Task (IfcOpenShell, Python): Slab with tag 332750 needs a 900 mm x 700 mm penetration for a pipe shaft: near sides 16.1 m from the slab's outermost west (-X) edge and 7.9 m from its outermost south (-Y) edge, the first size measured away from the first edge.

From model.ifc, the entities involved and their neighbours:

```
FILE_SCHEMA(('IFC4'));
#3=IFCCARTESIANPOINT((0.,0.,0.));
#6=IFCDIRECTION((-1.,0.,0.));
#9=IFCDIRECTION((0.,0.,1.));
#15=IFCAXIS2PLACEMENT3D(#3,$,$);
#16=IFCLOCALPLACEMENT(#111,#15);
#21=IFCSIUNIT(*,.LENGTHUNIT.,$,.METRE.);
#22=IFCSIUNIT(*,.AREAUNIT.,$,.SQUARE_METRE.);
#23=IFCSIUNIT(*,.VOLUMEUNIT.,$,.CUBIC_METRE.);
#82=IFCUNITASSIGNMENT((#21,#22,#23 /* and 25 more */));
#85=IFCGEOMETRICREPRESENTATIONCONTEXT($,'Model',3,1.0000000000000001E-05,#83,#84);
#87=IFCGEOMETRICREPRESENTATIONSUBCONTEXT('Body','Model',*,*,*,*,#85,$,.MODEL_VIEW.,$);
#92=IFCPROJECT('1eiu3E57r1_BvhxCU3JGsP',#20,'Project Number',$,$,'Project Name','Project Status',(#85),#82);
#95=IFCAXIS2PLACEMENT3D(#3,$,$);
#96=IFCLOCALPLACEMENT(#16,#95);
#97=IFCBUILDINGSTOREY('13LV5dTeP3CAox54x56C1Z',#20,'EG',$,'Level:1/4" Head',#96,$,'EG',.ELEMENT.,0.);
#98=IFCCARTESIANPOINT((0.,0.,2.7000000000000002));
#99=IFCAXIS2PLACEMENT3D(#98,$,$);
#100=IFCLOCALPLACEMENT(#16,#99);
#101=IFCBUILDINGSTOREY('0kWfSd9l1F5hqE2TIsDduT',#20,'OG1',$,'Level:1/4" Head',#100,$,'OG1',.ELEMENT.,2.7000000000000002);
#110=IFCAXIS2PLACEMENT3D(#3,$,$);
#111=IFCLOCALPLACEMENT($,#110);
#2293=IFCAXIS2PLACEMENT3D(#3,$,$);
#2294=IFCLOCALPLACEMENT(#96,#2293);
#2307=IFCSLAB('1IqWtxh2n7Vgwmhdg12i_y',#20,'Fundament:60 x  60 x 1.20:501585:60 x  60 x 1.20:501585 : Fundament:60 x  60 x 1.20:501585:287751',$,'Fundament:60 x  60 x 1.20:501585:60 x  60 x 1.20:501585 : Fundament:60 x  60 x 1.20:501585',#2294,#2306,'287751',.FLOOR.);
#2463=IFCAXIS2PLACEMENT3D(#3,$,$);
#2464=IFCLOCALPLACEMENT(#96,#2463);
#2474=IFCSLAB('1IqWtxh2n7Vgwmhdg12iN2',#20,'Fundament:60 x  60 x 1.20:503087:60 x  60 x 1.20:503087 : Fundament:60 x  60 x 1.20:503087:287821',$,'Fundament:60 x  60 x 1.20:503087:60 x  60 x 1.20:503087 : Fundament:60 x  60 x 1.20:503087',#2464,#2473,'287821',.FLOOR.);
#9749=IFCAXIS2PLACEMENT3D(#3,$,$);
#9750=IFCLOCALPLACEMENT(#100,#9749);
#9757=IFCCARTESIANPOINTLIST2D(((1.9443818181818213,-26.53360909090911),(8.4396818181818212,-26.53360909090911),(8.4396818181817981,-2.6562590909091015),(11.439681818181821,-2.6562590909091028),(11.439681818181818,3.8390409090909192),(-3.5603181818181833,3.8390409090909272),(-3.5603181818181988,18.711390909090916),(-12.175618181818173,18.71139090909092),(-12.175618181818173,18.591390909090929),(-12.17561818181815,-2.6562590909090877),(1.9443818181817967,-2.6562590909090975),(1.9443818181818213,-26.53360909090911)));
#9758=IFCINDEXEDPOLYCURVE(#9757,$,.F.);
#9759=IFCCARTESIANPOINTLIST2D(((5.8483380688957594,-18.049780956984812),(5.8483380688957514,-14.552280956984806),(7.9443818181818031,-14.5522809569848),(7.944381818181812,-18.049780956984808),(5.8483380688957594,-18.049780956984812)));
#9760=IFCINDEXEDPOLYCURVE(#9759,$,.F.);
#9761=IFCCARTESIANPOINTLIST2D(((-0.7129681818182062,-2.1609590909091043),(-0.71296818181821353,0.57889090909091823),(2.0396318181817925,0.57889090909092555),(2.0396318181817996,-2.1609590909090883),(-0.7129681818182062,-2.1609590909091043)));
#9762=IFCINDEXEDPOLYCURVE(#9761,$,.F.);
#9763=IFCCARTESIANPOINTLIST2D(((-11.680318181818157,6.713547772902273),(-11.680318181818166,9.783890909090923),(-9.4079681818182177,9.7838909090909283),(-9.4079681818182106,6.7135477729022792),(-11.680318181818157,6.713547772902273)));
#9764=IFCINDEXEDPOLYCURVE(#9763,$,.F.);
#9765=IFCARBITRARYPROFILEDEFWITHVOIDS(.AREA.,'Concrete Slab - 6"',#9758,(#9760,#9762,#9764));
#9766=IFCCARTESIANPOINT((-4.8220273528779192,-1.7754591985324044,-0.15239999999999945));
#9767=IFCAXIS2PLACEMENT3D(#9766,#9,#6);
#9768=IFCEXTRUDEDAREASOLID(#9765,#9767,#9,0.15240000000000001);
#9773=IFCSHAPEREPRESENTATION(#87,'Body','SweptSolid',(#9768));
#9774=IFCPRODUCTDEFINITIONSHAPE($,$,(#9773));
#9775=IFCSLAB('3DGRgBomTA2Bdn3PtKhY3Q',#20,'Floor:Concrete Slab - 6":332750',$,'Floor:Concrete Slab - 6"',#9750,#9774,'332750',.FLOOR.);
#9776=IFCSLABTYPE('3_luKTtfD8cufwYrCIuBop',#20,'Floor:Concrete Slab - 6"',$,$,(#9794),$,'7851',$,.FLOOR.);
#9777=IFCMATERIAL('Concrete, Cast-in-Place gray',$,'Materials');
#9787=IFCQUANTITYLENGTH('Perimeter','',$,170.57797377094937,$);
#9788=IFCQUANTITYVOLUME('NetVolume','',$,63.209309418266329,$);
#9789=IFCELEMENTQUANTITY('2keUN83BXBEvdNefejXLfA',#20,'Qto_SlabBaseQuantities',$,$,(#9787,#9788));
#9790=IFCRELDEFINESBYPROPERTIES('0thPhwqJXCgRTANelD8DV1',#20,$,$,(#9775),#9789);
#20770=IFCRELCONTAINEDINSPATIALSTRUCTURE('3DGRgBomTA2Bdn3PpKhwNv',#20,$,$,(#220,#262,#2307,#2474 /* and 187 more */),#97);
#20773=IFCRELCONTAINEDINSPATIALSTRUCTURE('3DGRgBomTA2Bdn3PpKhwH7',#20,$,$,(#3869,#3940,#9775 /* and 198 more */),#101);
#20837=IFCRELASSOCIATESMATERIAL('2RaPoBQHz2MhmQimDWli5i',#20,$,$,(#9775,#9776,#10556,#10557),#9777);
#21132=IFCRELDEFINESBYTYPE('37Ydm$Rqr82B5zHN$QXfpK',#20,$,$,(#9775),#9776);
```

```python
import numpy as np
import ifcopenshell
import ifcopenshell.api.feature
import ifcopenshell.api.geometry
import ifcopenshell.api.pset
import ifcopenshell.api.root
import ifcopenshell.geom
import ifcopenshell.util.element
import ifcopenshell.util.placement
import ifcopenshell.util.representation
import ifcopenshell.util.shape
import ifcopenshell.util.unit

model = ifcopenshell.open("model.ifc")
unit_scale = ifcopenshell.util.unit.calculate_unit_scale(model)
volume_scale = ifcopenshell.util.unit.calculate_unit_scale(model, "VOLUMEUNIT")
settings = ifcopenshell.geom.settings()


def volume(element):
    """Net volume in cubic metres, openings subtracted."""
    shape = ifcopenshell.geom.create_shape(settings, element)
    return ifcopenshell.util.shape.get_volume(shape.geometry)


slab = model.by_guid("3DGRgBomTA2Bdn3PtKhY3Q")
before = volume(slab)

# Extent in the slab's own axes, in metres. The edges named are its -X and -Y sides.
slab_shape = ifcopenshell.geom.create_shape(settings, slab)
vertices = ifcopenshell.util.shape.get_vertices(slab_shape.geometry)
x_min, y_min, bottom = vertices.min(axis=0)
top = vertices[:, 2].max()

opening = ifcopenshell.api.root.create_entity(model, ifc_class="IfcOpeningElement", name="Pipe shaft opening", predefined_type="OPENING")
context = ifcopenshell.util.representation.get_context(model, "Model", "Body", "MODEL_VIEW")
width, depth = 0.9, 0.7
outline = [(0.0, 0.0), (width, 0.0), (width, depth), (0.0, depth), (0.0, 0.0)]
# Overshoot both faces by 50 mm so the cut is clean.
shape = ifcopenshell.api.geometry.add_slab_representation(
    model, context=context, depth=top - bottom + 0.1, polyline=outline
)
ifcopenshell.api.geometry.assign_representation(model, product=opening, representation=shape)

matrix = ifcopenshell.util.placement.get_local_placement(slab.ObjectPlacement)
matrix[:, 3] = matrix @ np.append(np.array([x_min + 16.1, y_min + 7.9, bottom - 0.05]) / unit_scale, 1.0)
ifcopenshell.api.geometry.edit_object_placement(model, product=opening, matrix=matrix, is_si=False)
ifcopenshell.api.feature.add_feature(model, feature=opening, element=slab)

after = volume(slab)

# Update the slab's stored quantities.
qto = model.by_id(ifcopenshell.util.element.get_pset(slab, "Qto_SlabBaseQuantities", should_inherit=False)["id"])
ifcopenshell.api.pset.edit_qto(model, qto=qto, properties={"NetVolume": after / volume_scale})

print(f"slab volume {before:.3f} -> {after:.3f} m3")

model.write("model-out.ifc")
```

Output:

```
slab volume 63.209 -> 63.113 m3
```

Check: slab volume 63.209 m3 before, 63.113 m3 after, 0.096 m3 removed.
